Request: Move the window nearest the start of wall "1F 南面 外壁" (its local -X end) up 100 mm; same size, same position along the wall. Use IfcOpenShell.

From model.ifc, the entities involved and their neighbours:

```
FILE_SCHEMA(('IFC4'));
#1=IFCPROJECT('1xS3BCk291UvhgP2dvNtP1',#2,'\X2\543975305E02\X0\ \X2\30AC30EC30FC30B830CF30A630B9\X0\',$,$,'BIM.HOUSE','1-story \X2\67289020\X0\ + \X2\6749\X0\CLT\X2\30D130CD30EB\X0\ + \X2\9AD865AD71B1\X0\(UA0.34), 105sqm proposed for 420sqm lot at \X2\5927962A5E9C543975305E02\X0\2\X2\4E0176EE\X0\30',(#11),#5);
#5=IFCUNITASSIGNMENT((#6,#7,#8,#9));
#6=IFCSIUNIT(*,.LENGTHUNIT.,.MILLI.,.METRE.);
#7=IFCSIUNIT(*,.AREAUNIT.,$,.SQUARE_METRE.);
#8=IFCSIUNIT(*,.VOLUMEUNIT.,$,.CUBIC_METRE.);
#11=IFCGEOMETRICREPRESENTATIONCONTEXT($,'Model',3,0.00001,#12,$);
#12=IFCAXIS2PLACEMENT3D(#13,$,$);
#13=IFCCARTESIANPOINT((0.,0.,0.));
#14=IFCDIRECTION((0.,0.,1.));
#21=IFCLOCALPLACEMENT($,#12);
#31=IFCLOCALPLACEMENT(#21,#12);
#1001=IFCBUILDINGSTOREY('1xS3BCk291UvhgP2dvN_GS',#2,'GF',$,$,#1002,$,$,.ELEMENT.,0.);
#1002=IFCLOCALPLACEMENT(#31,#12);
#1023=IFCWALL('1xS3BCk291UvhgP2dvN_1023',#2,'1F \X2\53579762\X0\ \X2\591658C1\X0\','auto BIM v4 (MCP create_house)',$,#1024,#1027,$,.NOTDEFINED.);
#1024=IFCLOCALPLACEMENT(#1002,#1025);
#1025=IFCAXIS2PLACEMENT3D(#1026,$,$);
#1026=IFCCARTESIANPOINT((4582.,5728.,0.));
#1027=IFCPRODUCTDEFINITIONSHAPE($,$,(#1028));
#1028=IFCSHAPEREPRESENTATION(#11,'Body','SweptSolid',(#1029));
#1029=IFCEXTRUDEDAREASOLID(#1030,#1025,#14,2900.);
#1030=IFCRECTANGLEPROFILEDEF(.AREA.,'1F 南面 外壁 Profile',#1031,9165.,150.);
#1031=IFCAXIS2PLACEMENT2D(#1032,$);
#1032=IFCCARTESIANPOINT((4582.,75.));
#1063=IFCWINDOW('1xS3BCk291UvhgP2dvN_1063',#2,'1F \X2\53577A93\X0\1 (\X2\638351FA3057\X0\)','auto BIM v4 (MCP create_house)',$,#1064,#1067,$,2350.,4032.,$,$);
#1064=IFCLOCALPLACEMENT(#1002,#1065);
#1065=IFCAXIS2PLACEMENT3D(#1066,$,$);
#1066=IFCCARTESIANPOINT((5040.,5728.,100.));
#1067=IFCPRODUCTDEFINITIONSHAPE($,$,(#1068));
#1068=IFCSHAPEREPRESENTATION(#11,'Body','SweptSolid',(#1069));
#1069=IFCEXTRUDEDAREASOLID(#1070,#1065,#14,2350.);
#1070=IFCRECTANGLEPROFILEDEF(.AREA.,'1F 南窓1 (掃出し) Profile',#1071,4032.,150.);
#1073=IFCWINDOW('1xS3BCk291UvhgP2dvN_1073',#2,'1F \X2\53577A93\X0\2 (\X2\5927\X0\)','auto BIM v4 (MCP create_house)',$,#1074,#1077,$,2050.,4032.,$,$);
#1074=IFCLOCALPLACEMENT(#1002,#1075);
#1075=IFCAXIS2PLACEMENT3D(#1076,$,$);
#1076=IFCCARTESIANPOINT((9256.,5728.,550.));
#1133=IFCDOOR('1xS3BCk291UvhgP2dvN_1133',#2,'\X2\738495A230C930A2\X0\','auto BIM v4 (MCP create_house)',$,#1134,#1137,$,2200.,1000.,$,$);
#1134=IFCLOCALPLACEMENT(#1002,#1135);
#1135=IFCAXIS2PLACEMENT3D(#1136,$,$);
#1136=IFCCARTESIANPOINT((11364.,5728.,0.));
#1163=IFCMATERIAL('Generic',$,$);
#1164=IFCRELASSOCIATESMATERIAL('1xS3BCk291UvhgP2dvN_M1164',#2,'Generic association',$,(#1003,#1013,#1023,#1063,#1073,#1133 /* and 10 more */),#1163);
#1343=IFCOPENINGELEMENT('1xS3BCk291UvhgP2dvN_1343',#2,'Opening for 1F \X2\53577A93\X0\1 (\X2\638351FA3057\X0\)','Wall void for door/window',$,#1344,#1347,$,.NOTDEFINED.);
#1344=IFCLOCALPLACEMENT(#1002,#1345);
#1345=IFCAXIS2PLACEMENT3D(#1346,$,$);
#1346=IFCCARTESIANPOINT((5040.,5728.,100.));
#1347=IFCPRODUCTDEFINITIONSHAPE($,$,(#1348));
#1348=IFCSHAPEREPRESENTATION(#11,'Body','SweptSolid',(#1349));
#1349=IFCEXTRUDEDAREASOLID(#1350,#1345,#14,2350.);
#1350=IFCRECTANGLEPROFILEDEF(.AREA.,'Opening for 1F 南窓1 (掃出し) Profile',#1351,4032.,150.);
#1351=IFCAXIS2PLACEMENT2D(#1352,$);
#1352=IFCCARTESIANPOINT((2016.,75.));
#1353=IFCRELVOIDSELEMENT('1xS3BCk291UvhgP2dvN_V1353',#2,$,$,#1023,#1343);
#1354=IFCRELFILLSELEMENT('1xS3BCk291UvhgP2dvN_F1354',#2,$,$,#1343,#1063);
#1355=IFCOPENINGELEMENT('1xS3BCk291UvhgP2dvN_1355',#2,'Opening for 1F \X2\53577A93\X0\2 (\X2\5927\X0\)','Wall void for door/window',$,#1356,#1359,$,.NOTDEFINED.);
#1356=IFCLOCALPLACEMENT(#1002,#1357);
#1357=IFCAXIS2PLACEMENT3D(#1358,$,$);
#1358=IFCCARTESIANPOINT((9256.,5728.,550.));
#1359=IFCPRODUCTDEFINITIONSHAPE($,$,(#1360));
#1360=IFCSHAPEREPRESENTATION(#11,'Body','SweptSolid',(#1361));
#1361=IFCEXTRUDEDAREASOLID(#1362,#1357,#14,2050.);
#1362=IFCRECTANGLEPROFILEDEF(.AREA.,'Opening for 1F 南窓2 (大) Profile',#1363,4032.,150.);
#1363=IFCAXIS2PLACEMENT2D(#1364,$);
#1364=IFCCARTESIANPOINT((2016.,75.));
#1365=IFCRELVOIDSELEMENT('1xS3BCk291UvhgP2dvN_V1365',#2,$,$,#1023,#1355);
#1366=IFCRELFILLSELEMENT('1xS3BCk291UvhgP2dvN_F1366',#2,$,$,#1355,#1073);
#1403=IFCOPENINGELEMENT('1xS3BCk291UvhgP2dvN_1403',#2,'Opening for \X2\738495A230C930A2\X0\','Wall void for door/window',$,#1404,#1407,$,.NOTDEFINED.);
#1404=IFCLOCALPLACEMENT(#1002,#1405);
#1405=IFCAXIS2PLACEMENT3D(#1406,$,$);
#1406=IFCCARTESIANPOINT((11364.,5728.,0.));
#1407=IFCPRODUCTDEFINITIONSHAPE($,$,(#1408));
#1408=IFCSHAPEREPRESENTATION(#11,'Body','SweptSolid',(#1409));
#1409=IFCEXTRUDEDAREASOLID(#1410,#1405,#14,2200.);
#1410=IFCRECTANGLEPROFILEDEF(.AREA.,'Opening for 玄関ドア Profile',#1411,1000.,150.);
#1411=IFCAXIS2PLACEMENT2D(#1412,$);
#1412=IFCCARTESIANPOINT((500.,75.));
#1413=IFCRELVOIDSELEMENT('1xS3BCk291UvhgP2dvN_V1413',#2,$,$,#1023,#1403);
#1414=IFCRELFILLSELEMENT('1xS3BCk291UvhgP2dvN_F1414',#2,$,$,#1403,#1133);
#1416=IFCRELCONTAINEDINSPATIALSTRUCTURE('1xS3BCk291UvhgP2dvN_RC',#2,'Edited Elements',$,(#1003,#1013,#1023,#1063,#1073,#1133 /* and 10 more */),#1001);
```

```python
import numpy as np
import ifcopenshell
import ifcopenshell.api.geometry
import ifcopenshell.util.placement
import ifcopenshell.util.unit

model = ifcopenshell.open("model.ifc")
unit_scale = ifcopenshell.util.unit.calculate_unit_scale(model)

window = model.by_guid("1xS3BCk291UvhgP2dvN_1063")
opening = window.FillsVoids[0].RelatingOpeningElement
dz = 0.1 / unit_scale

shift = np.array([0.0, 0.0, dz])
# The window is not placed relative to its opening, so move both.
for product in (opening, window):
    matrix = ifcopenshell.util.placement.get_local_placement(product.ObjectPlacement)
    matrix[:3, 3] += shift
    ifcopenshell.api.geometry.edit_object_placement(model, product=product, matrix=matrix, is_si=False)

print(f"moved by {dz * unit_scale:+.3f} m")

model.write("model_rev.ifc")
```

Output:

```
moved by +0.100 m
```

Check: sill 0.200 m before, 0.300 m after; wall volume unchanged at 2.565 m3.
